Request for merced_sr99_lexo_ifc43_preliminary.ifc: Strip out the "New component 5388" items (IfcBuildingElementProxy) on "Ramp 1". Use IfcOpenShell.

First a look at what the model holds.

```python
import ifcopenshell
import ifcopenshell.util.element

model = ifcopenshell.open("merced_sr99_lexo_ifc43_preliminary.ifc")
print(model.schema)
storey = next(s for s in model.by_type("IfcBuildingStorey") if s.Name == "Ramp 1")
proxies = [e for e in ifcopenshell.util.element.get_decomposition(storey) if e.is_a("IfcBuildingElementProxy")]
seen = {}
for e in proxies:
    element_type = ifcopenshell.util.element.get_type(e)
    name = element_type.Name if element_type not in (None, e) else None
    seen[name] = seen.get(name, 0) + 1
for name, count in sorted(seen.items(), key=str):
    print(count, "x", name)
```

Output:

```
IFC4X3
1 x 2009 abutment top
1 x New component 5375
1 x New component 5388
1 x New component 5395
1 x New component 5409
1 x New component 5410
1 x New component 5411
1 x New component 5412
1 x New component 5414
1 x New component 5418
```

```python
import ifcopenshell
import ifcopenshell.api.root
import ifcopenshell.util.element

model = ifcopenshell.open("merced_sr99_lexo_ifc43_preliminary.ifc")

storey = next(s for s in model.by_type("IfcBuildingStorey") if s.Name == "Ramp 1")
proxies = [e for e in ifcopenshell.util.element.get_decomposition(storey) if e.is_a("IfcBuildingElementProxy")]
targets = [e for e in proxies if (t := ifcopenshell.util.element.get_type(e)) not in (None, e) and t.Name == "New component 5388"]

for e in targets:
    ifcopenshell.api.root.remove_product(model, product=e)
print(len(targets), "removed")

model.write("merced_sr99_lexo_ifc43_preliminary_updated.ifc")
```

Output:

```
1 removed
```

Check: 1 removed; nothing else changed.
